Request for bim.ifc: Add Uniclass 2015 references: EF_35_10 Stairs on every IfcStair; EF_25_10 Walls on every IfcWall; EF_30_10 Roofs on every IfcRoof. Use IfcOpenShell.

First a look at what the model holds.

```python
import ifcopenshell

model = ifcopenshell.open("bim.ifc")
print(model.schema)
print("classifications:", [c.Name for c in model.by_type("IfcClassification")])
for ifc_class in ("IfcDoor", "IfcRoof", "IfcStair", "IfcWall", "IfcWindow"):
    print(ifc_class, len(model.by_type(ifc_class)))
```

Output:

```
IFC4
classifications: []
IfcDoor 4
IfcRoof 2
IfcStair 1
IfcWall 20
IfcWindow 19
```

```python
import ifcopenshell
import ifcopenshell.api.classification

model = ifcopenshell.open("bim.ifc")

system = ifcopenshell.api.classification.add_classification(model, classification="Uniclass 2015")

codes = {
    "IfcStair": ("EF_35_10", "Stairs"),
    "IfcWall": ("EF_25_10", "Walls"),
    "IfcRoof": ("EF_30_10", "Roofs"),
}
for ifc_class, (code, name) in codes.items():
    products = model.by_type(ifc_class)
    ifcopenshell.api.classification.add_reference(
        model, products=products, classification=system, identification=code, name=name
    )
    print(code, len(products))

model.write("bim_edited.ifc")
```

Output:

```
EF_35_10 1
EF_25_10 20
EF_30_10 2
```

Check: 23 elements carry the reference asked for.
